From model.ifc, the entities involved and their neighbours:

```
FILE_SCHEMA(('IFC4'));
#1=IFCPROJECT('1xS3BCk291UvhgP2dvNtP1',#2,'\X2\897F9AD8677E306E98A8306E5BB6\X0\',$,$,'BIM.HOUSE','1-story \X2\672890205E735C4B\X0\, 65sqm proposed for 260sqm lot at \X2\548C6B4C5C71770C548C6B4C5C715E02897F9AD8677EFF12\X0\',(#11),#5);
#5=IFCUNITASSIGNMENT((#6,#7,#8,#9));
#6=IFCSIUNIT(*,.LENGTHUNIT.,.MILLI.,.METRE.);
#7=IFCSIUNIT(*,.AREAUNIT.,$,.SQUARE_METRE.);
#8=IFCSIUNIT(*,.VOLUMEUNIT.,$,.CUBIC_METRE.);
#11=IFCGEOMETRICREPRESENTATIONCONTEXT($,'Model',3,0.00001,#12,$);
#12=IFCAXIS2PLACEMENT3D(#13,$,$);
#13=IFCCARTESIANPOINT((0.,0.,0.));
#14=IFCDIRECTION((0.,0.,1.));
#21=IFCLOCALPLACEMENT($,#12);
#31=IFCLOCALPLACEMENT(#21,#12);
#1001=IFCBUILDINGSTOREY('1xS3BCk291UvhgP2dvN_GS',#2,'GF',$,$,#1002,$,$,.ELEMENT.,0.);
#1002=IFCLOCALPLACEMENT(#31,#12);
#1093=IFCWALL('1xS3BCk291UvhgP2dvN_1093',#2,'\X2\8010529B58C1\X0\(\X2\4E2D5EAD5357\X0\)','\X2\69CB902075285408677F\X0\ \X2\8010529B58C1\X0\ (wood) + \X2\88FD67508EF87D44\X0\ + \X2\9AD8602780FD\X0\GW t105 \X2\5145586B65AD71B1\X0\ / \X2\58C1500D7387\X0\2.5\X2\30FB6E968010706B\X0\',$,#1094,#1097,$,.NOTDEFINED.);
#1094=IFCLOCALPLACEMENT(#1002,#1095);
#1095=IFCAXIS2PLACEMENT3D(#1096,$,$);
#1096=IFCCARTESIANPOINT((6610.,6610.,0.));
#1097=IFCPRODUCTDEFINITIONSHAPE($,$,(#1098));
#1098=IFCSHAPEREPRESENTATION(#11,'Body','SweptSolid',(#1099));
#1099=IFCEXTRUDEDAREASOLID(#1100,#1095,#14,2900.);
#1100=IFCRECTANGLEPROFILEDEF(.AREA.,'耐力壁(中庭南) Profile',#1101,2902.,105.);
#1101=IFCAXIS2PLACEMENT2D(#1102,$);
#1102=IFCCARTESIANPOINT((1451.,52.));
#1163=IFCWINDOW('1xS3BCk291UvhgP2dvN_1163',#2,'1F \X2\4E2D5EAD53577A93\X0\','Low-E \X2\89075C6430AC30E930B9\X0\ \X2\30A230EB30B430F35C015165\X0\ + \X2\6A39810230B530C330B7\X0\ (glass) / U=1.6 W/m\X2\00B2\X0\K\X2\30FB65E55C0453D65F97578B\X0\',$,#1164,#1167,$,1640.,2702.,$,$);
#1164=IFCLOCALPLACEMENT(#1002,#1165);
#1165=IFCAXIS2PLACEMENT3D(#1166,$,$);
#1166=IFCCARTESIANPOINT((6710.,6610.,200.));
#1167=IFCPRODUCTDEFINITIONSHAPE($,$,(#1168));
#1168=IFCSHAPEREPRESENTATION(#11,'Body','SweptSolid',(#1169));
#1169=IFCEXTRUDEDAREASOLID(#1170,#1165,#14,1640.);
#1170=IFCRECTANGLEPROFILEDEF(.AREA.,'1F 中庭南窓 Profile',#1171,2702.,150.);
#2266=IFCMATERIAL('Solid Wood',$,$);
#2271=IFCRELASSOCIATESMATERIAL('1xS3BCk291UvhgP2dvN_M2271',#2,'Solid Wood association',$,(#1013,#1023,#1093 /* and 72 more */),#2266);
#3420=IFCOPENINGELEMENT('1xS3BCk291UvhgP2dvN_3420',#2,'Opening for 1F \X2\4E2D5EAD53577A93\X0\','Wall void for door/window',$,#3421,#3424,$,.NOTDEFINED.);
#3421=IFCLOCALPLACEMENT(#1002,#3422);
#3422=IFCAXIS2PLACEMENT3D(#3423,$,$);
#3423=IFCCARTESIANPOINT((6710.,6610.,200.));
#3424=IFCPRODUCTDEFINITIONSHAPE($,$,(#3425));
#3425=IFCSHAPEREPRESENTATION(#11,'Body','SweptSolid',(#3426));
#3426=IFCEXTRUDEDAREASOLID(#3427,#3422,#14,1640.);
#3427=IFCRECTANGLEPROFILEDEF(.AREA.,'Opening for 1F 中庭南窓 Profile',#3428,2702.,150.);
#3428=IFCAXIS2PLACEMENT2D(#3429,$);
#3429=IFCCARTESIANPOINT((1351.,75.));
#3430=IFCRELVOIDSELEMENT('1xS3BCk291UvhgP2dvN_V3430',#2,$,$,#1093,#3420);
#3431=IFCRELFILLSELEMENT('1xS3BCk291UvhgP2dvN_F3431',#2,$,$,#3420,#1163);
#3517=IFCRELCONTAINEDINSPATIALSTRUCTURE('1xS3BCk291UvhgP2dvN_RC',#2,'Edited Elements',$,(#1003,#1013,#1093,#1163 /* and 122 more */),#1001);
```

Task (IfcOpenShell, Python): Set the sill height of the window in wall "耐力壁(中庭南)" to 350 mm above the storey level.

```python
import numpy as np
import ifcopenshell
import ifcopenshell.api.geometry
import ifcopenshell.geom
import ifcopenshell.util.element
import ifcopenshell.util.placement
import ifcopenshell.util.shape
import ifcopenshell.util.unit

model = ifcopenshell.open("model.ifc")
unit_scale = ifcopenshell.util.unit.calculate_unit_scale(model)

window = model.by_guid("1xS3BCk291UvhgP2dvN_1163")
opening = window.FillsVoids[0].RelatingOpeningElement
storey = ifcopenshell.util.element.get_container(window, ifc_class="IfcBuildingStorey")
level = ifcopenshell.util.placement.get_local_placement(storey.ObjectPlacement)[2, 3]

# The opening's origin need not be at the sill, so measure its lowest point.
shape = ifcopenshell.geom.create_shape(ifcopenshell.geom.settings(), opening)
bottom = ifcopenshell.util.shape.get_shape_bottom_elevation(shape, shape.geometry) / unit_scale
dz = level + 0.35 / unit_scale - bottom

shift = np.array([0.0, 0.0, dz])
# The window is not placed relative to its opening, so move both.
for product in (opening, window):
    matrix = ifcopenshell.util.placement.get_local_placement(product.ObjectPlacement)
    matrix[:3, 3] += shift
    ifcopenshell.api.geometry.edit_object_placement(model, product=product, matrix=matrix, is_si=False)

print(f"moved by {dz * unit_scale:+.3f} m")

model.write("model_updated.ifc")
```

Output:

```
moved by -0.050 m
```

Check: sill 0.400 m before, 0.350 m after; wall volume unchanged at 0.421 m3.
